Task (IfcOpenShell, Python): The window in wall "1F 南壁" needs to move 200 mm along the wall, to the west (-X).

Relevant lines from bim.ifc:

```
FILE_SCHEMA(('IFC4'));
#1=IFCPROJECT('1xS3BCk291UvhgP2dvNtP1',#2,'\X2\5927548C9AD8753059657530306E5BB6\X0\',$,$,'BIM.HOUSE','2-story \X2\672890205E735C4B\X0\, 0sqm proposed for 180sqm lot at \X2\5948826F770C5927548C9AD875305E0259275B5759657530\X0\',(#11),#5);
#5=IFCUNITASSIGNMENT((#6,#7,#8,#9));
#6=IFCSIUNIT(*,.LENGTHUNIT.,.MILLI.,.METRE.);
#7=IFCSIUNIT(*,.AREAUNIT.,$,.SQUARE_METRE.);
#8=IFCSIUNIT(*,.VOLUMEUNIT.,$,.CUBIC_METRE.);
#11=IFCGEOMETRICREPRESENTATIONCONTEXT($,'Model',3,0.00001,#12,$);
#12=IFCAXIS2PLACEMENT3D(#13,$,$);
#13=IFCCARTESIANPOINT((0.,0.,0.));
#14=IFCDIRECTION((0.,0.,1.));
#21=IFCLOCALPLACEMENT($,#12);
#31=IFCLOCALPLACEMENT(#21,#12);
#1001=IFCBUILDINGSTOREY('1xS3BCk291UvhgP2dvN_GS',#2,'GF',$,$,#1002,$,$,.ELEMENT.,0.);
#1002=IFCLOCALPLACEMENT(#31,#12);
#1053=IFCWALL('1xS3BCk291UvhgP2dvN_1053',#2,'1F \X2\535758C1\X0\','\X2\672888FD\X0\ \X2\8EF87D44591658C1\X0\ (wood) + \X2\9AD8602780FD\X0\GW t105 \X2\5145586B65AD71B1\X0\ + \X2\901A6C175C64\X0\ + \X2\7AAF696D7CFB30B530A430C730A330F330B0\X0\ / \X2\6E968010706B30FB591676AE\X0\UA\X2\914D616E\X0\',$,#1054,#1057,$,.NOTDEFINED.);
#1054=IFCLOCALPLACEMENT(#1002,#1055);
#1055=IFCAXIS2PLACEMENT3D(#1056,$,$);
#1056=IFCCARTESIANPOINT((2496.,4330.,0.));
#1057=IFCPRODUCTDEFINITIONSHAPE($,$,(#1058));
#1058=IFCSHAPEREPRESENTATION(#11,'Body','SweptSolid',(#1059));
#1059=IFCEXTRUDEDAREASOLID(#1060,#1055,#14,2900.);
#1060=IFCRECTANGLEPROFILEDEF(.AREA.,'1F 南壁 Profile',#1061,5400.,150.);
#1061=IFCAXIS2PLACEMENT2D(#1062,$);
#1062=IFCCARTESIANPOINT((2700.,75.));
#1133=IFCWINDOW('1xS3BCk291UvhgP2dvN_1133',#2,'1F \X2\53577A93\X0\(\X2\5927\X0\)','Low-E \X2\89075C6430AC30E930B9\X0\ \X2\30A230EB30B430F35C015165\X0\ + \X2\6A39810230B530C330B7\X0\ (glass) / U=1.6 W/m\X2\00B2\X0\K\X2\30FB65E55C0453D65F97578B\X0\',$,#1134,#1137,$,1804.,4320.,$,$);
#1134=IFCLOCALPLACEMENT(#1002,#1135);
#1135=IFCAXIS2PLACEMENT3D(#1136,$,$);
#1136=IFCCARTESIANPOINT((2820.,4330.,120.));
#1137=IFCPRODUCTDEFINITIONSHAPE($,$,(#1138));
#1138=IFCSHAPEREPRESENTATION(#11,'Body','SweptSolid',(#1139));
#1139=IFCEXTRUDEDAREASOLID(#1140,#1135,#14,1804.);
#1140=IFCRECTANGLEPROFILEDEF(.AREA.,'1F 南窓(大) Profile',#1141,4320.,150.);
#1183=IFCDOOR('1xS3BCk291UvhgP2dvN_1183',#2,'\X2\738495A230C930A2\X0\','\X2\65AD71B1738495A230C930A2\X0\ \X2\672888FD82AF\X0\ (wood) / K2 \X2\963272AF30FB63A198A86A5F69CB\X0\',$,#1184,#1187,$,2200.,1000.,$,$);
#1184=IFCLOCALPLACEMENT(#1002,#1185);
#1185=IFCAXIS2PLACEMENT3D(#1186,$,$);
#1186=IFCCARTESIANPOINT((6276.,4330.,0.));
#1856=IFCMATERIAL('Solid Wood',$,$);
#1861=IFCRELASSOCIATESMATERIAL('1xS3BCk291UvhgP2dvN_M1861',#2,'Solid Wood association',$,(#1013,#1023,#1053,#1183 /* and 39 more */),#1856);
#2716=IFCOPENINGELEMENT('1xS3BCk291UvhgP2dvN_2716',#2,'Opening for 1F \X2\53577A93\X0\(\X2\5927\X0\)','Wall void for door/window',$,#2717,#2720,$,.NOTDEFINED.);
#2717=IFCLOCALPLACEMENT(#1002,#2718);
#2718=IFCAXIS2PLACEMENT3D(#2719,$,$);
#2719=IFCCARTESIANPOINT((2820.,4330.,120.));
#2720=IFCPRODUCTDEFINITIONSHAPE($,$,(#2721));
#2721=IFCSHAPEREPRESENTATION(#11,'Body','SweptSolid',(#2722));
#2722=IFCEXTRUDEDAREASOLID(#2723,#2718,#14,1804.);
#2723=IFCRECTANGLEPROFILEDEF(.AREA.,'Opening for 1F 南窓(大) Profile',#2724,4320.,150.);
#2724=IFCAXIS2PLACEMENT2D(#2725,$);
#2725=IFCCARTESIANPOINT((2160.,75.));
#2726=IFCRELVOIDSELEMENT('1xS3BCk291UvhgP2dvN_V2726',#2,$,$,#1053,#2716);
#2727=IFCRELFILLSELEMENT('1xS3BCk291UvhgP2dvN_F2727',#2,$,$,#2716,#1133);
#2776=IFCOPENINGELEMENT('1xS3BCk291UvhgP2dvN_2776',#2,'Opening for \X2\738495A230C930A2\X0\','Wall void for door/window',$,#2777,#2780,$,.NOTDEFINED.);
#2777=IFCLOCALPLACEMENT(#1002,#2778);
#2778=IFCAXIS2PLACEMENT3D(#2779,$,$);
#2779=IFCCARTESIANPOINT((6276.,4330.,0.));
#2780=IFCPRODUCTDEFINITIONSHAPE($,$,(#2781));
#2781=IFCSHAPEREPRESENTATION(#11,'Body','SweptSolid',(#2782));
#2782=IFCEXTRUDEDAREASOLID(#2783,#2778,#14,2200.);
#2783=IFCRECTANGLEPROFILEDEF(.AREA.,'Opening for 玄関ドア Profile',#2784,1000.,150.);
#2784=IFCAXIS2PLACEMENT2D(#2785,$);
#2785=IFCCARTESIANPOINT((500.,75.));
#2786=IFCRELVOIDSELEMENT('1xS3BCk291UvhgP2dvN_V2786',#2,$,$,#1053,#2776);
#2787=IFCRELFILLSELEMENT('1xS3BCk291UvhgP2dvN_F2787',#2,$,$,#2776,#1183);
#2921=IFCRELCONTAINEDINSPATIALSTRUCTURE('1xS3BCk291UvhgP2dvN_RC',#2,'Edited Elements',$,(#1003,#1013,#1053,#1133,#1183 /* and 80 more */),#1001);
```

```python
import ifcopenshell
import ifcopenshell.api.geometry
import ifcopenshell.util.placement
import ifcopenshell.util.unit

model = ifcopenshell.open("bim.ifc")
unit_scale = ifcopenshell.util.unit.calculate_unit_scale(model)

window = model.by_guid("1xS3BCk291UvhgP2dvN_1133")
opening = window.FillsVoids[0].RelatingOpeningElement
wall = opening.VoidsElements[0].RelatingBuildingElement

wall_matrix = ifcopenshell.util.placement.get_local_placement(wall.ObjectPlacement)
shift = wall_matrix[:3, 0] * -0.2 / unit_scale
before = ifcopenshell.util.placement.get_local_placement(window.ObjectPlacement)[:3, 3].copy()

# The window is not placed relative to its opening, so move both.
for product in (opening, window):
    matrix = ifcopenshell.util.placement.get_local_placement(product.ObjectPlacement)
    matrix[:3, 3] += shift
    ifcopenshell.api.geometry.edit_object_placement(model, product=product, matrix=matrix, is_si=False)

after = ifcopenshell.util.placement.get_local_placement(window.ObjectPlacement)[:3, 3]
print("window moved by", (after - before).round(3) + 0.0)

model.write("bim_rev.ifc")
```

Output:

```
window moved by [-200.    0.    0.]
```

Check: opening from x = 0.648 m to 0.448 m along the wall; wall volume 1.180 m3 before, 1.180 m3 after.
